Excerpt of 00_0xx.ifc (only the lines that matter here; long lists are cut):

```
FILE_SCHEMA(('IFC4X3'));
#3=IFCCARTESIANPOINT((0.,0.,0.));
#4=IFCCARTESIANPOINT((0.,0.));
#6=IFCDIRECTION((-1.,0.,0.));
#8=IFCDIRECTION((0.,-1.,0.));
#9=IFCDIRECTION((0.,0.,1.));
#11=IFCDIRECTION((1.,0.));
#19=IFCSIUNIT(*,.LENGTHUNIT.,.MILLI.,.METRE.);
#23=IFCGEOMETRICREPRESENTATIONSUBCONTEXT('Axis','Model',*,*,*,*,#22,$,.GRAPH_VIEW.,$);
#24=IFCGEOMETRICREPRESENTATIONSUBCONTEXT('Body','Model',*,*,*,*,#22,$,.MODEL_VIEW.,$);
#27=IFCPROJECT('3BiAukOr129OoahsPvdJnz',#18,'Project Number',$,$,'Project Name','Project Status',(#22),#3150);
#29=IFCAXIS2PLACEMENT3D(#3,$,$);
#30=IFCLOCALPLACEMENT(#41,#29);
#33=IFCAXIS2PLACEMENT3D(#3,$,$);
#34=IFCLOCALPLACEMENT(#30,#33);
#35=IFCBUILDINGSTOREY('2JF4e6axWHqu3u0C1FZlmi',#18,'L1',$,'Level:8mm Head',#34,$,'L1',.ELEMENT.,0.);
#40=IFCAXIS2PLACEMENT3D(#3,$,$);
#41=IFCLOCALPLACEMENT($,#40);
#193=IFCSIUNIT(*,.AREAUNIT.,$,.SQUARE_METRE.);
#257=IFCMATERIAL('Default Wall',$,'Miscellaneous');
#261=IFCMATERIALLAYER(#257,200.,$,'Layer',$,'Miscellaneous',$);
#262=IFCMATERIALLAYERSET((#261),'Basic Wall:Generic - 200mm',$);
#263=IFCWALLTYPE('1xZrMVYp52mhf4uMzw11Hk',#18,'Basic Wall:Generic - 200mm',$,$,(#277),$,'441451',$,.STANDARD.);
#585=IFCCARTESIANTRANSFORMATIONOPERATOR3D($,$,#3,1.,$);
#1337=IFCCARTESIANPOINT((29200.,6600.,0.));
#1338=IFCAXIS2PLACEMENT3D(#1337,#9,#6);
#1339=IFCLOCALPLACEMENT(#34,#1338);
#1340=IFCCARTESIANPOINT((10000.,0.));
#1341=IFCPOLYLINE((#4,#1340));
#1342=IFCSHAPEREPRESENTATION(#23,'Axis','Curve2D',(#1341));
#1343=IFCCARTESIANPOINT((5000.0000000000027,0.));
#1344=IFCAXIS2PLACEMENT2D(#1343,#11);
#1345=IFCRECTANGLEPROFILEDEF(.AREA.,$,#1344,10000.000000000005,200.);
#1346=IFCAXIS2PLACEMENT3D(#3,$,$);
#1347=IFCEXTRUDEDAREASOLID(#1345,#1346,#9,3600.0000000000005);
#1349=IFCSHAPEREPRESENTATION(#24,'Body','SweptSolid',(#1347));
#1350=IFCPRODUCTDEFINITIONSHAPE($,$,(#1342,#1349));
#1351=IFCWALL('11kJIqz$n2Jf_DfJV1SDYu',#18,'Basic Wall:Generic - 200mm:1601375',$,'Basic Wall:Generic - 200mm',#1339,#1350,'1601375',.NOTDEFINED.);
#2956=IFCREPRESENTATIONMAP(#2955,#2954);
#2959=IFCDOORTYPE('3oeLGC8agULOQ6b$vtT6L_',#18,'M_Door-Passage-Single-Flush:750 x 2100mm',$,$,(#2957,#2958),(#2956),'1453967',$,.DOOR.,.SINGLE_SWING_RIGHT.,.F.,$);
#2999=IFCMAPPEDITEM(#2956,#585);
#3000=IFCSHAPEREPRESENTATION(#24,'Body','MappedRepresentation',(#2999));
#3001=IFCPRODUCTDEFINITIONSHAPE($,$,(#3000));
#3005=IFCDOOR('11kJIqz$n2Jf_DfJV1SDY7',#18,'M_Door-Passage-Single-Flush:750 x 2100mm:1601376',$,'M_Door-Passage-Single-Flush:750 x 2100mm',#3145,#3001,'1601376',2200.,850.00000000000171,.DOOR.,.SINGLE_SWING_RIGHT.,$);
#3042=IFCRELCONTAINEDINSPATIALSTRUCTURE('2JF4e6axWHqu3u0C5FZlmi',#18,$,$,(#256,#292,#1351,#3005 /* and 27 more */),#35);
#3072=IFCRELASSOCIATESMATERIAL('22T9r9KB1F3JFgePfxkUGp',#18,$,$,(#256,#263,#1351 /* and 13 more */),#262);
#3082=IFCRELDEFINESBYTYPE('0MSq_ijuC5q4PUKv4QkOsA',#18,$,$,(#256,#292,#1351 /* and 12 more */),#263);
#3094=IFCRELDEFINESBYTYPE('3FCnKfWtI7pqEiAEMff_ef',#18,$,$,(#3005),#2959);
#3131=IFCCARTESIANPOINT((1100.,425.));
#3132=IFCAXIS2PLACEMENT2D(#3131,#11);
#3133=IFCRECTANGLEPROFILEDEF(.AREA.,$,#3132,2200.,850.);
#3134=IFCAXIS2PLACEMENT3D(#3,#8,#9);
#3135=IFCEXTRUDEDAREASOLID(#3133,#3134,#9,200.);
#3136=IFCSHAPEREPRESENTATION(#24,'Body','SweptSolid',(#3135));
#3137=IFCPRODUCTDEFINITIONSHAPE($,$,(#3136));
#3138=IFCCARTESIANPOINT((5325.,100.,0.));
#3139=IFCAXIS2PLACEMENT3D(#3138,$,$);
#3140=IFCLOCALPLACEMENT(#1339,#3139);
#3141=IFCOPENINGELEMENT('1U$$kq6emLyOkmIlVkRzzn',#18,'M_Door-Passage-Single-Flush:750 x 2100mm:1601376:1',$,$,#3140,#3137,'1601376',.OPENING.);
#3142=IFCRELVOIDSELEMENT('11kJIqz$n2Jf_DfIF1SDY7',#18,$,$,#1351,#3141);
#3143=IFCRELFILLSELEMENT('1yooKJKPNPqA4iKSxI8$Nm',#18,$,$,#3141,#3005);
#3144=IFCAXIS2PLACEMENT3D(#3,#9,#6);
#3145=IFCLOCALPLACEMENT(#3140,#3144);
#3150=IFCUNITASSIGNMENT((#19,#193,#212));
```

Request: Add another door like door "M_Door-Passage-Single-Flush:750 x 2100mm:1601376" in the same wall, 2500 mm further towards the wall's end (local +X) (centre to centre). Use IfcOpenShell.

```python
import ifcopenshell
import ifcopenshell.api.feature
import ifcopenshell.api.geometry
import ifcopenshell.api.root
import ifcopenshell.geom
import ifcopenshell.util.element
import ifcopenshell.util.placement
import ifcopenshell.util.shape

model = ifcopenshell.open("00_0xx.ifc")
settings = ifcopenshell.geom.settings()


def volume(element):
    """Net volume in cubic metres, openings subtracted."""
    shape = ifcopenshell.geom.create_shape(settings, element)
    return ifcopenshell.util.shape.get_volume(shape.geometry)


def reuse_history(source, copy):
    """copy_class also copies each property set's owner history, people and application; keep the originals."""
    for rel in copy.IsDefinedBy:
        if rel.is_a("IfcRelDefinesByProperties") and (history := rel.RelatingPropertyDefinition.OwnerHistory):
            rel.RelatingPropertyDefinition.OwnerHistory = source.OwnerHistory
            ifcopenshell.util.element.remove_deep2(model, history)


door = model.by_guid("11kJIqz$n2Jf_DfJV1SDY7")
opening = door.FillsVoids[0].RelatingOpeningElement
wall = opening.VoidsElements[0].RelatingBuildingElement
before = volume(wall)
shift = ifcopenshell.util.placement.get_local_placement(wall.ObjectPlacement)[:3, 0] * 2500.0

# copy_class copies the void relationship, type, container and properties, but no geometry.
new_opening = ifcopenshell.api.root.copy_class(model, product=opening)
new_opening.Representation = ifcopenshell.util.element.copy_deep(
    model, opening.Representation, exclude=["IfcGeometricRepresentationContext", "IfcRepresentationMap"]
)
new_opening.Name = "M_Door-Passage-Single-Flush:750 x 2100mm"
new_opening.Tag = None
new_door = ifcopenshell.api.root.copy_class(model, product=door)
new_door.Representation = ifcopenshell.util.element.copy_deep(
    model, door.Representation, exclude=["IfcGeometricRepresentationContext", "IfcRepresentationMap"]
)
new_door.Name = "M_Door-Passage-Single-Flush:750 x 2100mm"
new_door.Tag = None
reuse_history(door, new_door)
ifcopenshell.api.feature.add_filling(model, opening=new_opening, element=new_door)

for old, new in ((opening, new_opening), (door, new_door)):
    matrix = ifcopenshell.util.placement.get_local_placement(old.ObjectPlacement)
    matrix[:3, 3] += shift
    ifcopenshell.api.geometry.edit_object_placement(model, product=new, matrix=matrix, is_si=False)

after = volume(wall)

print(f"wall volume {before:.3f} -> {after:.3f} m3")

model.write("00_0xx_edited.ifc")
```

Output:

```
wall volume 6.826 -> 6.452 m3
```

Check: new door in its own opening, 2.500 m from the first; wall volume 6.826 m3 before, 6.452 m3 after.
